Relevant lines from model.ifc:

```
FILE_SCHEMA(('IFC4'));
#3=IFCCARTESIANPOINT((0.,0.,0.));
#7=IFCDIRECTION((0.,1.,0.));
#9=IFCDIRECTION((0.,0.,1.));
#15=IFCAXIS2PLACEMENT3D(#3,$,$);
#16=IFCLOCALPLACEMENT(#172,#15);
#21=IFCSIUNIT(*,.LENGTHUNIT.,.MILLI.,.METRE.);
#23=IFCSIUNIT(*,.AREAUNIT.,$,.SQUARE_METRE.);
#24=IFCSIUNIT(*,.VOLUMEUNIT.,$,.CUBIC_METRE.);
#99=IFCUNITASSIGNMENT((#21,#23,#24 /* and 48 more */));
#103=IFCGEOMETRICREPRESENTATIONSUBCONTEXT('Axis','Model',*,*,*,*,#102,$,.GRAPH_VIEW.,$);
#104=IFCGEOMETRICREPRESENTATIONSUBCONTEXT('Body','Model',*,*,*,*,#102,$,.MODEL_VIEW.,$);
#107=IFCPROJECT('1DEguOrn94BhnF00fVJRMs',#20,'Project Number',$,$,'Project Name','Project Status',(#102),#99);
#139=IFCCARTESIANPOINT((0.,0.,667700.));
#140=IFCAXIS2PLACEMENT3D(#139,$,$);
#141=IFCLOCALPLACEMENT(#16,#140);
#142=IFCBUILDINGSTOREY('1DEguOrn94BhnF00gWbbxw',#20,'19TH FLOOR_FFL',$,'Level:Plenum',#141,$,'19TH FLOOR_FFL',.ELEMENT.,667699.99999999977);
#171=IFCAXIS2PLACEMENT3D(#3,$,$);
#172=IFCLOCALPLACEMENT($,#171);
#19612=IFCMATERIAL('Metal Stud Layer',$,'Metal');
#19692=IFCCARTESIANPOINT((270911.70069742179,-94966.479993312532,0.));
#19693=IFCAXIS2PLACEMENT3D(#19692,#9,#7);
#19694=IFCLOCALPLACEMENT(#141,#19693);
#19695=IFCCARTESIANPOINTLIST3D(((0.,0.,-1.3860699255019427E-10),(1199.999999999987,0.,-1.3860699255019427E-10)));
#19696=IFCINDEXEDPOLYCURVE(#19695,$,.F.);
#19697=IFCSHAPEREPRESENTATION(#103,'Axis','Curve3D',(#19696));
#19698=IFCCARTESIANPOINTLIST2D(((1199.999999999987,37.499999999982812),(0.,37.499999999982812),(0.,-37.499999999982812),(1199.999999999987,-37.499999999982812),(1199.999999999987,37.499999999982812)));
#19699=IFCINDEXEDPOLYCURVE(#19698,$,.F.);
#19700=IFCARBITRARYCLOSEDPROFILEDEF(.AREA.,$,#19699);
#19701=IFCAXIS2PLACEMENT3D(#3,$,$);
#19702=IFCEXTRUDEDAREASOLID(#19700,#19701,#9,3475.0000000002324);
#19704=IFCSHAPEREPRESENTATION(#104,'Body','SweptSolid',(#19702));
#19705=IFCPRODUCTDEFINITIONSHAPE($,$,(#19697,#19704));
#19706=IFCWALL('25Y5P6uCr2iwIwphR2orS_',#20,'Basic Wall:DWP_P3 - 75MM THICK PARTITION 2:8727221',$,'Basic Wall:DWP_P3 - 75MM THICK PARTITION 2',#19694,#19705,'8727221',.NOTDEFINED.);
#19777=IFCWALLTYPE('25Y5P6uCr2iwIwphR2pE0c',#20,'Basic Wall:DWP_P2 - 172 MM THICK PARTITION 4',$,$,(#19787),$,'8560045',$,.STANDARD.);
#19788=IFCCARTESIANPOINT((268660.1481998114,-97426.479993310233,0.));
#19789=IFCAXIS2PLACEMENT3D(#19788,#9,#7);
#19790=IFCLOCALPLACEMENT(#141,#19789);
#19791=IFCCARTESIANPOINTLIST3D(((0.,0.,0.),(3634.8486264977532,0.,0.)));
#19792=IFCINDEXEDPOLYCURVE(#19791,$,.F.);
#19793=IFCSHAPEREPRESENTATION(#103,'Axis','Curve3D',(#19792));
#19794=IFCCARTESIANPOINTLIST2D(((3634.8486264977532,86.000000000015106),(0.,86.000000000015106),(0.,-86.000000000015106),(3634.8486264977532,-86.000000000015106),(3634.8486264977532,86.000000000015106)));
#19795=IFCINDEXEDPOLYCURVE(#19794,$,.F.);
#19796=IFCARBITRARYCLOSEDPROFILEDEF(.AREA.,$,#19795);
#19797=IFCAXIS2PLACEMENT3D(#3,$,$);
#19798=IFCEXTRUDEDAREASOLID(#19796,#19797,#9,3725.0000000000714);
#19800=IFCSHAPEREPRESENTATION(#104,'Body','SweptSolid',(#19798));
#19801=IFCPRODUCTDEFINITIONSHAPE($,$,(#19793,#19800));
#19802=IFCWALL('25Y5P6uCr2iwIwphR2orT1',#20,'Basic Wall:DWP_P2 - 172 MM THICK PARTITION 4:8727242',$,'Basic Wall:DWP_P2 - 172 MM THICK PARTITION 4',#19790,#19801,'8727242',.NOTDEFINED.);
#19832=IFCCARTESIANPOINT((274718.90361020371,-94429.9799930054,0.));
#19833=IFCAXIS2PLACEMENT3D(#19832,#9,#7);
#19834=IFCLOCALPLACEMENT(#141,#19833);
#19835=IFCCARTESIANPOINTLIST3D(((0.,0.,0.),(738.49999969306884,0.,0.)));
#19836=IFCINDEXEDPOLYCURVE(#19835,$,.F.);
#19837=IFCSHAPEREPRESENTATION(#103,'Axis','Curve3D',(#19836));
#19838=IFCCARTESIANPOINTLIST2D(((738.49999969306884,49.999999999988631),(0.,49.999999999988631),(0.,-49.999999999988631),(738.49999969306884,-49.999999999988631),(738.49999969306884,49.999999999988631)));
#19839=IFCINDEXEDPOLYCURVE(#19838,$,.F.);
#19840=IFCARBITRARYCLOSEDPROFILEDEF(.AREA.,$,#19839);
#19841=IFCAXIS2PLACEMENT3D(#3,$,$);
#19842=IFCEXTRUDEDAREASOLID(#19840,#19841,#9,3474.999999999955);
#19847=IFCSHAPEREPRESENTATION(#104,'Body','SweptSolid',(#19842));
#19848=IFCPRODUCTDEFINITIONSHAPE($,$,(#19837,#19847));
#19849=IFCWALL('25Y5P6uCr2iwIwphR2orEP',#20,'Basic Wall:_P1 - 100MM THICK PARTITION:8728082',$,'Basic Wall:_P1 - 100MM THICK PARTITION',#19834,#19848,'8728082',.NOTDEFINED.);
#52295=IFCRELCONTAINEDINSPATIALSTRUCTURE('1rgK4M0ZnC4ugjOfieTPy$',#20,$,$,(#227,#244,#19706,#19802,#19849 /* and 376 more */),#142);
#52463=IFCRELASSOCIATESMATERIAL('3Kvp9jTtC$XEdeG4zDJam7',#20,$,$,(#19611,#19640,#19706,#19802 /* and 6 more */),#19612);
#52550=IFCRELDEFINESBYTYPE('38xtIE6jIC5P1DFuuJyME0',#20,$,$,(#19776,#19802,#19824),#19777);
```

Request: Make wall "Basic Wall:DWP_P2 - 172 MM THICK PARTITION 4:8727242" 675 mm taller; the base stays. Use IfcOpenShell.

```python
import ifcopenshell
import ifcopenshell.geom
import ifcopenshell.util.representation
import ifcopenshell.util.shape
import ifcopenshell.util.unit

model = ifcopenshell.open("model.ifc")
unit_scale = ifcopenshell.util.unit.calculate_unit_scale(model)
settings = ifcopenshell.geom.settings()


def volume(element):
    """Net volume in cubic metres, openings subtracted."""
    shape = ifcopenshell.geom.create_shape(settings, element)
    return ifcopenshell.util.shape.get_volume(shape.geometry)


wall = model.by_id(19802)
before = volume(wall)

body = ifcopenshell.util.representation.get_representation(wall, "Model", "Body")
solid = body.Items[0]
old_height = solid.Depth
solid.Depth += 0.675 / unit_scale
after = volume(wall)

print(f"height {old_height:g} -> {solid.Depth:g}, volume {before:.3f} -> {after:.3f} m3")

model.write("model_v2.ifc")
```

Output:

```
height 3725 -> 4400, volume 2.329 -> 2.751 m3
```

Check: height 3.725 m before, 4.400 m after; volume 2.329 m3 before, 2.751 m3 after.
